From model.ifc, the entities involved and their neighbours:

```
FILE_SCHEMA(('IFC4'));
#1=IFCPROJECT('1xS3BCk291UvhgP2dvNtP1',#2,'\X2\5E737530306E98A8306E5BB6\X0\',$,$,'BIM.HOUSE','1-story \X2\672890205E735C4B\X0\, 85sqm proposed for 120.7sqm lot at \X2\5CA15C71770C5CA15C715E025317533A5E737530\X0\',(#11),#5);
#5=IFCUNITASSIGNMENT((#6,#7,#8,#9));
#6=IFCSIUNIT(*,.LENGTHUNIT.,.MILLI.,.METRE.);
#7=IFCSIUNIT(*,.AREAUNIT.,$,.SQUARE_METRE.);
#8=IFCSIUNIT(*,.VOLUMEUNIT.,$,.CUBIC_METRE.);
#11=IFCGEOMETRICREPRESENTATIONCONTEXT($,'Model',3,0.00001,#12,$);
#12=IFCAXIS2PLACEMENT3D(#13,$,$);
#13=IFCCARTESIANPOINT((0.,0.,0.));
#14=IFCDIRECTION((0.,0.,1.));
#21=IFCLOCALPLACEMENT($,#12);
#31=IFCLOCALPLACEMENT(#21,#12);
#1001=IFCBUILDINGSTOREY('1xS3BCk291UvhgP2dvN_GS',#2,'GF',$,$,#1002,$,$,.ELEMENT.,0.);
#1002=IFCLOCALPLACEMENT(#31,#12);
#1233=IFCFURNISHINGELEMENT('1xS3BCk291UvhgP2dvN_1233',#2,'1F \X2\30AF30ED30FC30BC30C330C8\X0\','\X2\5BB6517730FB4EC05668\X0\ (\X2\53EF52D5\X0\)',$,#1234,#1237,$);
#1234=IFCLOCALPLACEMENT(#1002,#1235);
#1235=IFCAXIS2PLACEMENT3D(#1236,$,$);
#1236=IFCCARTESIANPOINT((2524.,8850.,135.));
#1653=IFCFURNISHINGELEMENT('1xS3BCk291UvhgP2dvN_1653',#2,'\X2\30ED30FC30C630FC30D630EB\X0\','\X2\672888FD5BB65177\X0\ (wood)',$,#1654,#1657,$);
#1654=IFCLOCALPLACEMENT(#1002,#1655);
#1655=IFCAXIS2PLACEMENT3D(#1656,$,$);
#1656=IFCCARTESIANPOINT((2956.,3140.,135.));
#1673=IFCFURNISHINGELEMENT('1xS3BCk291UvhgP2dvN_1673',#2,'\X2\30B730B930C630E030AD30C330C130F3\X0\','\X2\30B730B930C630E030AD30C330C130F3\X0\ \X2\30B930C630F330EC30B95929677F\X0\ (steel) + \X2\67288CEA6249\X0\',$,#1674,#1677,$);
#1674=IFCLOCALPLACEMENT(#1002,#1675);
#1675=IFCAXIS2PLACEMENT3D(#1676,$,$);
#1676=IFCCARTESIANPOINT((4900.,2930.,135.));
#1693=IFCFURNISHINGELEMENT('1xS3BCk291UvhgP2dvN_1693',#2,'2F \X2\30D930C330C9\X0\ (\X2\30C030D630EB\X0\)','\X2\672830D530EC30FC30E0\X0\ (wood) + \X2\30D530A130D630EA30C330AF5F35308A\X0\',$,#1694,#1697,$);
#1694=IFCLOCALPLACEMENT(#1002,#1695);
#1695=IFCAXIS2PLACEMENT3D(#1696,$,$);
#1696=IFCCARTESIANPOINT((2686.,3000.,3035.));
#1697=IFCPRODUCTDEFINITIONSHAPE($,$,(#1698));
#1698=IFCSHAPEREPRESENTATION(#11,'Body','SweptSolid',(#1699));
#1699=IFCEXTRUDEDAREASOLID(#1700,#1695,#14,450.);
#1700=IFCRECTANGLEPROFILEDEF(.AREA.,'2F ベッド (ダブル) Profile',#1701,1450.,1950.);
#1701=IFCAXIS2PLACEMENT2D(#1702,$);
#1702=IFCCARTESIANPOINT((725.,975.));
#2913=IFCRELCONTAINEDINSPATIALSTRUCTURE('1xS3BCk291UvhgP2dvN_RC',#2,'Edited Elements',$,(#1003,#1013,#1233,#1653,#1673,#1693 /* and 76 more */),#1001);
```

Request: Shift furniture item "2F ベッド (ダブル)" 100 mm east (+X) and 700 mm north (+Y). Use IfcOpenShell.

```python
import ifcopenshell
import ifcopenshell.api.geometry
import ifcopenshell.util.placement
import ifcopenshell.util.unit

model = ifcopenshell.open("model.ifc")
unit_scale = ifcopenshell.util.unit.calculate_unit_scale(model)

item = model.by_guid("1xS3BCk291UvhgP2dvN_1693")
matrix = ifcopenshell.util.placement.get_local_placement(item.ObjectPlacement)
matrix[0, 3] += 0.1 / unit_scale
matrix[1, 3] += 0.7 / unit_scale
ifcopenshell.api.geometry.edit_object_placement(model, product=item, matrix=matrix, is_si=False)

print(ifcopenshell.util.placement.get_local_placement(item.ObjectPlacement).round(3) + 0.0)

model.write("model-out.ifc")
```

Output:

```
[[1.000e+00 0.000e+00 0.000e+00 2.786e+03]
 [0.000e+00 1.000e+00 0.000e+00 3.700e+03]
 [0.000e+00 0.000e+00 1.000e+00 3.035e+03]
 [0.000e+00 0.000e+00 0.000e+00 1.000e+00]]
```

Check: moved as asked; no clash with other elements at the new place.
